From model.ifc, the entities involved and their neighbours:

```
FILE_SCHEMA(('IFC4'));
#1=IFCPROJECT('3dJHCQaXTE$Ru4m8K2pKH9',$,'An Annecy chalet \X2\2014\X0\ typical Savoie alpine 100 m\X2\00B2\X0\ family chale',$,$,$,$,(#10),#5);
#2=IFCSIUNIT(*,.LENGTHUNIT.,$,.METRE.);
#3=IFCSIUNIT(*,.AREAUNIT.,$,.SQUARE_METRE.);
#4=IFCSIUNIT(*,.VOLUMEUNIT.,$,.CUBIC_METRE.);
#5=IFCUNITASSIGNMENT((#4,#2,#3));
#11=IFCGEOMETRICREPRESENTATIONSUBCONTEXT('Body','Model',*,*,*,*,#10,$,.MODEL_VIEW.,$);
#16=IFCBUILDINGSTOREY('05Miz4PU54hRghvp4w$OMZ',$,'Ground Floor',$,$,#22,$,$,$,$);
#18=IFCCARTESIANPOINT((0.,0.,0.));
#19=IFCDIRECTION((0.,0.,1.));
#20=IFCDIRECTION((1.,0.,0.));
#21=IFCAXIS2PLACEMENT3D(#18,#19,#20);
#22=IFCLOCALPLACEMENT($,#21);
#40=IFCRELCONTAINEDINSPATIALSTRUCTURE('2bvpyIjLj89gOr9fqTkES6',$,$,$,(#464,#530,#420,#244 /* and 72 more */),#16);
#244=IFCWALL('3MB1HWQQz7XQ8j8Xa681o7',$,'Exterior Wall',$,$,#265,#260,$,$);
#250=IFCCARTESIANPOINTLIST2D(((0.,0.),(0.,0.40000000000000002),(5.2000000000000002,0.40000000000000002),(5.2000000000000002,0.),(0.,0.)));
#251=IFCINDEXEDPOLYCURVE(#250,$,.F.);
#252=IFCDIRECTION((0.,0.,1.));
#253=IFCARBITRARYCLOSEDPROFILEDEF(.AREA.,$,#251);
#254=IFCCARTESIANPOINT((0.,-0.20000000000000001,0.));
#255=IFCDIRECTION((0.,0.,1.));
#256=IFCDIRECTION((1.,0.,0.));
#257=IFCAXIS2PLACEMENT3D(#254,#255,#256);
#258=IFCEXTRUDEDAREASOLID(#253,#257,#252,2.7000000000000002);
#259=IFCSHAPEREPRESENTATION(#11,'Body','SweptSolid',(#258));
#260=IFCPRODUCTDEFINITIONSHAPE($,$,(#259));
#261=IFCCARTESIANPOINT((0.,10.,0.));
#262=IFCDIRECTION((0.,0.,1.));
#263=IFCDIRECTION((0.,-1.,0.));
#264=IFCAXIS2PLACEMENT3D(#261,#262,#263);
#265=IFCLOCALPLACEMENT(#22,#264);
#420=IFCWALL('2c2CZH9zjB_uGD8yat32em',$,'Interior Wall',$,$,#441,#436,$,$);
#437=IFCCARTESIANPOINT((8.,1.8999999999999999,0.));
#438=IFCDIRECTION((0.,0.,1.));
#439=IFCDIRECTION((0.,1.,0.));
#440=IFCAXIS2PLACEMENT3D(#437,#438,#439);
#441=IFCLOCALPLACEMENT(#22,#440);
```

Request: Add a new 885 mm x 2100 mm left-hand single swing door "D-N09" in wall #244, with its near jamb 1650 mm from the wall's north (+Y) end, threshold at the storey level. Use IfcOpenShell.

```python
import numpy as np
import ifcopenshell
import ifcopenshell.api.feature
import ifcopenshell.api.geometry
import ifcopenshell.api.root
import ifcopenshell.api.spatial
import ifcopenshell.geom
import ifcopenshell.util.element
import ifcopenshell.util.placement
import ifcopenshell.util.representation
import ifcopenshell.util.shape
import ifcopenshell.util.unit

model = ifcopenshell.open("model.ifc")
unit_scale = ifcopenshell.util.unit.calculate_unit_scale(model)
settings = ifcopenshell.geom.settings()


def volume(element):
    """Net volume in cubic metres, openings subtracted."""
    shape = ifcopenshell.geom.create_shape(settings, element)
    return ifcopenshell.util.shape.get_volume(shape.geometry)


wall = model.by_guid("3MB1HWQQz7XQ8j8Xa681o7")
storey = ifcopenshell.util.element.get_container(wall, ifc_class="IfcBuildingStorey")
context = ifcopenshell.util.representation.get_context(model, "Model", "Body", "MODEL_VIEW")
before = volume(wall)

width, height, from_end, sill = 0.885, 2.1, 1.65, 0.0  # metres

# The wall runs along its own X axis, and the end named is its -X end.
wall_shape = ifcopenshell.geom.create_shape(settings, wall)
x, y, z = ifcopenshell.util.shape.get_vertices(wall_shape.geometry).T
start = x.min() + from_end
face, thickness = float(y.min()), float(y.max() - y.min())
wall_matrix = ifcopenshell.util.placement.get_local_placement(wall.ObjectPlacement)
level = ifcopenshell.util.placement.get_local_placement(storey.ObjectPlacement)[2, 3]


def in_wall(x, y):
    """Placement at x, y metres in the wall's axes, at sill height."""
    matrix = wall_matrix.copy()
    matrix[:, 3] = wall_matrix @ np.array([x / unit_scale, y / unit_scale, 0.0, 1.0])
    matrix[2, 3] = level + sill / unit_scale
    return matrix


# Opening: a box that overshoots both wall faces by 50 mm.
opening = ifcopenshell.api.root.create_entity(model, ifc_class="IfcOpeningElement", predefined_type="OPENING")
box = ifcopenshell.api.geometry.add_wall_representation(
    model, context=context, length=width, height=height, thickness=thickness + 0.1
)
ifcopenshell.api.geometry.assign_representation(model, product=opening, representation=box)
ifcopenshell.api.geometry.edit_object_placement(model, product=opening, matrix=in_wall(start, face - 0.05), is_si=False)
ifcopenshell.api.feature.add_feature(model, feature=opening, element=wall)

door = ifcopenshell.api.root.create_entity(model, ifc_class="IfcDoor", name="D-N09", predefined_type="DOOR")
door.OverallWidth, door.OverallHeight = width / unit_scale, height / unit_scale
door.OperationType = "SINGLE_SWING_LEFT"
body = ifcopenshell.api.geometry.add_door_representation(
    model,
    context=context,
    overall_width=door.OverallWidth,
    overall_height=door.OverallHeight,
    operation_type="SINGLE_SWING_LEFT",
    lining_properties={"LiningDepth": thickness / unit_scale, "ThresholdDepth": thickness / unit_scale},
)
ifcopenshell.api.geometry.assign_representation(model, product=door, representation=body)
ifcopenshell.api.spatial.assign_container(model, products=[door], relating_structure=storey)
ifcopenshell.api.feature.add_filling(model, opening=opening, element=door)

# The lining spans the wall, so the door starts at the wall face.
ifcopenshell.api.geometry.edit_object_placement(model, product=door, matrix=in_wall(start, face), is_si=False)

after = volume(wall)

print(f"wall volume {before:.3f} -> {after:.3f} m3")

model.write("model_updated.ifc")
```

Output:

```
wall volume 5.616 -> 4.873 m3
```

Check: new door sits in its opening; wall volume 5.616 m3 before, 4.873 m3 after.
